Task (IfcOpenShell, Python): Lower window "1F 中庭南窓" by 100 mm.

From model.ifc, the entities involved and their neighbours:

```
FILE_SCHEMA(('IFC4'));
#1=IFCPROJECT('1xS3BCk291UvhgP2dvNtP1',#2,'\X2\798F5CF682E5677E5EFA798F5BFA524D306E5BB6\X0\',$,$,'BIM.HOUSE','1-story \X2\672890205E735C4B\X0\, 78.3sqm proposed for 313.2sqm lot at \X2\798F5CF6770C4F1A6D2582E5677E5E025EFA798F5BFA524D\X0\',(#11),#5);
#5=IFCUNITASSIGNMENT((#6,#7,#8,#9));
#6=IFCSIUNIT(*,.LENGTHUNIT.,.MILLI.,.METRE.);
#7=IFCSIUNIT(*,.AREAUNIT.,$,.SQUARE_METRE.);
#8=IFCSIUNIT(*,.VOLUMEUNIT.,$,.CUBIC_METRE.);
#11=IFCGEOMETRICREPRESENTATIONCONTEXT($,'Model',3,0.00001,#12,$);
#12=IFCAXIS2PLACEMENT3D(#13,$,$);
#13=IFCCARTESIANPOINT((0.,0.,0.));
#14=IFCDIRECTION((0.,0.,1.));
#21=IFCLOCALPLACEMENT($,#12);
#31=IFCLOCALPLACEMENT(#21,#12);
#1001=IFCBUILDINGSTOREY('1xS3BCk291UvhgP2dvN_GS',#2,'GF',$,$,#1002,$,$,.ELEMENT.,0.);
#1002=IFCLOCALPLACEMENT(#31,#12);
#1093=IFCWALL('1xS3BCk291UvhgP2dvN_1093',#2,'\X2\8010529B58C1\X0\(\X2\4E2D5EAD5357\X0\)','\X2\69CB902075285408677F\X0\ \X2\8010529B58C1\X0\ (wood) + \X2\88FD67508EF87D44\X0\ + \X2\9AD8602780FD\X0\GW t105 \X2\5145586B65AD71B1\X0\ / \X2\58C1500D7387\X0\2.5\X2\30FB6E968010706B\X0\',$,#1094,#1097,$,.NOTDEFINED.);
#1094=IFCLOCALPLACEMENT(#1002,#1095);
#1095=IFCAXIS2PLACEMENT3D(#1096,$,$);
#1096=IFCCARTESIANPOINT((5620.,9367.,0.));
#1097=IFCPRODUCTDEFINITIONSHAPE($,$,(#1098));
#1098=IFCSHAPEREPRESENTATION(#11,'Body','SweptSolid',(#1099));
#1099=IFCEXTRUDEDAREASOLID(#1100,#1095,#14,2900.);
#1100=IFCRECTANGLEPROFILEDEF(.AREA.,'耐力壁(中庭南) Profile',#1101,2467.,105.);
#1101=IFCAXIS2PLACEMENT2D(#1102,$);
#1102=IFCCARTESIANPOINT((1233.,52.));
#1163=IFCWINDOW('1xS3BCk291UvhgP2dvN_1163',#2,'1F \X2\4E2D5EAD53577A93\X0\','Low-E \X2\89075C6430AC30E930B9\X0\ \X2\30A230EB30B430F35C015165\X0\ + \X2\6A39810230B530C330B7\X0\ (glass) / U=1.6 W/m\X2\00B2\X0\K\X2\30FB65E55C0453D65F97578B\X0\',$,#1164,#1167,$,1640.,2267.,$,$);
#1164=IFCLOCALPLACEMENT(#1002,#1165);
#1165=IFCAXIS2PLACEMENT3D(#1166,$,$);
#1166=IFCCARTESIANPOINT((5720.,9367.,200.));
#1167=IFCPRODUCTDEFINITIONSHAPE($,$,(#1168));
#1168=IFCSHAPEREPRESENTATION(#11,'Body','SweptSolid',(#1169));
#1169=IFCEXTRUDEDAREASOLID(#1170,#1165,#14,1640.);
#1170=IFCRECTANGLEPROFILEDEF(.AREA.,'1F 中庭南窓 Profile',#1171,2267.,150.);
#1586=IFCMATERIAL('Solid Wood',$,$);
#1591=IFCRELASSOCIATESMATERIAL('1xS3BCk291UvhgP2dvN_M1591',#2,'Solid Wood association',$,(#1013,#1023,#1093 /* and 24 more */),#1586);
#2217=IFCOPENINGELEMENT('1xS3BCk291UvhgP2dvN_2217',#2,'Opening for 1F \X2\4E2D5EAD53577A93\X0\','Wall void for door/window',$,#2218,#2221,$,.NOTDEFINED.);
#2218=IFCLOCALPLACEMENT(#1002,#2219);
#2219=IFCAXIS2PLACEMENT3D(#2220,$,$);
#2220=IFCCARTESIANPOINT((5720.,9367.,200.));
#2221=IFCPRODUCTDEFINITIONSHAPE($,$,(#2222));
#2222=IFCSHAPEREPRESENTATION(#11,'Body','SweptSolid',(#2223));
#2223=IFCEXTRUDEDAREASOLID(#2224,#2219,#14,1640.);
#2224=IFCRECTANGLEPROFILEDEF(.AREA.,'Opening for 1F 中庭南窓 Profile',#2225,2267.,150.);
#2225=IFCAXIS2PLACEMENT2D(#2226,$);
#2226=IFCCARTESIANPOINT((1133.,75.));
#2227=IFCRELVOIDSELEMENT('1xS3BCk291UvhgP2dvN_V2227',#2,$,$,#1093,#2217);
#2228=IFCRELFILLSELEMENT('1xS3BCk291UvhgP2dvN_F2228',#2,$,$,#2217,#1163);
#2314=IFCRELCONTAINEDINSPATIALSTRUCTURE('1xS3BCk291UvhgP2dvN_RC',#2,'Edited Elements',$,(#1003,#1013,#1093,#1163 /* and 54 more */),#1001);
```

```python
import numpy as np
import ifcopenshell
import ifcopenshell.api.geometry
import ifcopenshell.util.placement
import ifcopenshell.util.unit

model = ifcopenshell.open("model.ifc")
unit_scale = ifcopenshell.util.unit.calculate_unit_scale(model)

window = model.by_guid("1xS3BCk291UvhgP2dvN_1163")
opening = window.FillsVoids[0].RelatingOpeningElement
dz = -0.1 / unit_scale

shift = np.array([0.0, 0.0, dz])
# The window is not placed relative to its opening, so move both.
for product in (opening, window):
    matrix = ifcopenshell.util.placement.get_local_placement(product.ObjectPlacement)
    matrix[:3, 3] += shift
    ifcopenshell.api.geometry.edit_object_placement(model, product=product, matrix=matrix, is_si=False)

print(f"moved by {dz * unit_scale:+.3f} m")

model.write("model_updated.ifc")
```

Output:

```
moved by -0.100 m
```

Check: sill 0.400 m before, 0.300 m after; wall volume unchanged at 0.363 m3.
